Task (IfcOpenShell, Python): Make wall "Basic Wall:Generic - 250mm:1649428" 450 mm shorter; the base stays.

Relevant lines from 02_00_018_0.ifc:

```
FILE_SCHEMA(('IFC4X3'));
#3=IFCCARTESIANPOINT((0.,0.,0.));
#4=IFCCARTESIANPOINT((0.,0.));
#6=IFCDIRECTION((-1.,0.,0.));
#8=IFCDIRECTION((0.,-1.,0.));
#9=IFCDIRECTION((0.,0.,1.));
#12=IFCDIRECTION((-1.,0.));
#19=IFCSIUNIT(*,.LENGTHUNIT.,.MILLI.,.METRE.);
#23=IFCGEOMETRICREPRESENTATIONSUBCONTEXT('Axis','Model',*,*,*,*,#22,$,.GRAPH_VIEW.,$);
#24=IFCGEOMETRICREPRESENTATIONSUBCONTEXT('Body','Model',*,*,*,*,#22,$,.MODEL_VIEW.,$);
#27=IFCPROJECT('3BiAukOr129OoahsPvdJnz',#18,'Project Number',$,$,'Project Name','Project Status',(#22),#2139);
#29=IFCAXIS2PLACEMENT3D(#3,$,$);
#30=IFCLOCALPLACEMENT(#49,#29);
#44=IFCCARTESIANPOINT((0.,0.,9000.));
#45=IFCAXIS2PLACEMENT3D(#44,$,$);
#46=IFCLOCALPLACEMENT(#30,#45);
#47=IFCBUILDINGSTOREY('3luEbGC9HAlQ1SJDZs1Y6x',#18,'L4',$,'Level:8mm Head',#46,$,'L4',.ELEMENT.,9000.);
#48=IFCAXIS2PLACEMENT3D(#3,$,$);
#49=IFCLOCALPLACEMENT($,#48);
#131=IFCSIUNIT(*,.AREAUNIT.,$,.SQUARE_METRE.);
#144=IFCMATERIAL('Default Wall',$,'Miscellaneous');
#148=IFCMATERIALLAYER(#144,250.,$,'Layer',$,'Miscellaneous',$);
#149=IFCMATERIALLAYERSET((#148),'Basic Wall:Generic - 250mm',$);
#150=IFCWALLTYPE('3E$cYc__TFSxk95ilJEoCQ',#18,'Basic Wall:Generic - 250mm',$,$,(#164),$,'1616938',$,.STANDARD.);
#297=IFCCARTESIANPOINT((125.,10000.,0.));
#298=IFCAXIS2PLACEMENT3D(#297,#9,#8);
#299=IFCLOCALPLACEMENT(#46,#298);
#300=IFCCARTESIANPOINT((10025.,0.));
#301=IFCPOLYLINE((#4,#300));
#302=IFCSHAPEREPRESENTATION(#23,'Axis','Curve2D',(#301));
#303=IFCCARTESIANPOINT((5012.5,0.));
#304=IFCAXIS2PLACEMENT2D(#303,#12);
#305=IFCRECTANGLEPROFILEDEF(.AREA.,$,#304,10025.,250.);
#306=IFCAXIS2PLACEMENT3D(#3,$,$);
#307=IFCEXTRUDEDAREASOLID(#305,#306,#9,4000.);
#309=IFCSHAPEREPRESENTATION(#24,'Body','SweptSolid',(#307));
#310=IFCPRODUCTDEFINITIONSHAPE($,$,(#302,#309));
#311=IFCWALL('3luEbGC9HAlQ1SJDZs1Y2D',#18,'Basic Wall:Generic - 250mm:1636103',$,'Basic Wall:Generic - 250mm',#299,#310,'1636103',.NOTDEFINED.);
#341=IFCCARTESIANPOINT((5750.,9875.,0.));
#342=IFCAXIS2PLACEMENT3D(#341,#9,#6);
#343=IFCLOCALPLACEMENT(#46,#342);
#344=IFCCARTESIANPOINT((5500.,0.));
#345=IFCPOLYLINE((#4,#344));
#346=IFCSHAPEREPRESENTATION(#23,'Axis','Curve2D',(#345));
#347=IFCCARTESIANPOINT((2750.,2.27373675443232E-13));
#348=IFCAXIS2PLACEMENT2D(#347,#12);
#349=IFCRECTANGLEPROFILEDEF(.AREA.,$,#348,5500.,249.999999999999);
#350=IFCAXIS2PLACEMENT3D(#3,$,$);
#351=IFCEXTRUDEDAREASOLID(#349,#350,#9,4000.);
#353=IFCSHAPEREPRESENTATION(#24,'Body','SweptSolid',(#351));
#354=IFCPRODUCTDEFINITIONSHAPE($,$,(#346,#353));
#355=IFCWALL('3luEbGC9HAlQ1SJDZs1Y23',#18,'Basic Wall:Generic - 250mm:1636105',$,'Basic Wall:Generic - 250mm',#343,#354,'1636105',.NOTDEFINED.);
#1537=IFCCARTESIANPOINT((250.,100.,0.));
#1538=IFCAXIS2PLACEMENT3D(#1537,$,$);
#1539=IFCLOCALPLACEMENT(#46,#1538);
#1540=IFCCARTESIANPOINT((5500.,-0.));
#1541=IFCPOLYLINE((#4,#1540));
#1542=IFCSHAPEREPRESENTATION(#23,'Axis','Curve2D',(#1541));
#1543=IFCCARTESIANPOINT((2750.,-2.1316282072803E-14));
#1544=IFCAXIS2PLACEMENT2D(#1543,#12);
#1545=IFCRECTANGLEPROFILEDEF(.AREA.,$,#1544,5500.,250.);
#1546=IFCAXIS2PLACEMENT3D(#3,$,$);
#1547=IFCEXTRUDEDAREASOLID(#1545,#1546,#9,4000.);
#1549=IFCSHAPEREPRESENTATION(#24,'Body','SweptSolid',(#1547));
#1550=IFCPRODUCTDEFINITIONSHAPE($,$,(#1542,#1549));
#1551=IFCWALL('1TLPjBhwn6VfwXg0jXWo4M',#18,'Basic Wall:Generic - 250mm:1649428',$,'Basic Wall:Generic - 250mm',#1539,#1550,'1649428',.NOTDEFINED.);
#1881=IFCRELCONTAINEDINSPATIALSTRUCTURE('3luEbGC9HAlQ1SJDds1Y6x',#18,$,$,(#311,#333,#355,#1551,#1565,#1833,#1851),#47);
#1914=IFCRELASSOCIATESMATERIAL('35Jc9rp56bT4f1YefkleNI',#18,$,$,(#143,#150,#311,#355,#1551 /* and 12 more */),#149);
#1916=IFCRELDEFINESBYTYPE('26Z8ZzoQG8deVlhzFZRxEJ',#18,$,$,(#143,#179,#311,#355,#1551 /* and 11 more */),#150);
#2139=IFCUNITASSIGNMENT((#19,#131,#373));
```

```python
import ifcopenshell
import ifcopenshell.geom
import ifcopenshell.util.representation
import ifcopenshell.util.shape

model = ifcopenshell.open("02_00_018_0.ifc")
settings = ifcopenshell.geom.settings()


def volume(element):
    """Net volume in cubic metres, openings subtracted."""
    shape = ifcopenshell.geom.create_shape(settings, element)
    return ifcopenshell.util.shape.get_volume(shape.geometry)


wall = model.by_guid("1TLPjBhwn6VfwXg0jXWo4M")
before = volume(wall)

body = ifcopenshell.util.representation.get_representation(wall, "Model", "Body")
solid = body.Items[0]
old_height = solid.Depth
solid.Depth -= 450.0
after = volume(wall)

print(f"height {old_height:g} -> {solid.Depth:g}, volume {before:.3f} -> {after:.3f} m3")

model.write("02_00_018_0_v2.ifc")
```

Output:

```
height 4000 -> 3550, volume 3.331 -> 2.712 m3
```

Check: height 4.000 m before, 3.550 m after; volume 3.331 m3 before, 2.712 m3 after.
